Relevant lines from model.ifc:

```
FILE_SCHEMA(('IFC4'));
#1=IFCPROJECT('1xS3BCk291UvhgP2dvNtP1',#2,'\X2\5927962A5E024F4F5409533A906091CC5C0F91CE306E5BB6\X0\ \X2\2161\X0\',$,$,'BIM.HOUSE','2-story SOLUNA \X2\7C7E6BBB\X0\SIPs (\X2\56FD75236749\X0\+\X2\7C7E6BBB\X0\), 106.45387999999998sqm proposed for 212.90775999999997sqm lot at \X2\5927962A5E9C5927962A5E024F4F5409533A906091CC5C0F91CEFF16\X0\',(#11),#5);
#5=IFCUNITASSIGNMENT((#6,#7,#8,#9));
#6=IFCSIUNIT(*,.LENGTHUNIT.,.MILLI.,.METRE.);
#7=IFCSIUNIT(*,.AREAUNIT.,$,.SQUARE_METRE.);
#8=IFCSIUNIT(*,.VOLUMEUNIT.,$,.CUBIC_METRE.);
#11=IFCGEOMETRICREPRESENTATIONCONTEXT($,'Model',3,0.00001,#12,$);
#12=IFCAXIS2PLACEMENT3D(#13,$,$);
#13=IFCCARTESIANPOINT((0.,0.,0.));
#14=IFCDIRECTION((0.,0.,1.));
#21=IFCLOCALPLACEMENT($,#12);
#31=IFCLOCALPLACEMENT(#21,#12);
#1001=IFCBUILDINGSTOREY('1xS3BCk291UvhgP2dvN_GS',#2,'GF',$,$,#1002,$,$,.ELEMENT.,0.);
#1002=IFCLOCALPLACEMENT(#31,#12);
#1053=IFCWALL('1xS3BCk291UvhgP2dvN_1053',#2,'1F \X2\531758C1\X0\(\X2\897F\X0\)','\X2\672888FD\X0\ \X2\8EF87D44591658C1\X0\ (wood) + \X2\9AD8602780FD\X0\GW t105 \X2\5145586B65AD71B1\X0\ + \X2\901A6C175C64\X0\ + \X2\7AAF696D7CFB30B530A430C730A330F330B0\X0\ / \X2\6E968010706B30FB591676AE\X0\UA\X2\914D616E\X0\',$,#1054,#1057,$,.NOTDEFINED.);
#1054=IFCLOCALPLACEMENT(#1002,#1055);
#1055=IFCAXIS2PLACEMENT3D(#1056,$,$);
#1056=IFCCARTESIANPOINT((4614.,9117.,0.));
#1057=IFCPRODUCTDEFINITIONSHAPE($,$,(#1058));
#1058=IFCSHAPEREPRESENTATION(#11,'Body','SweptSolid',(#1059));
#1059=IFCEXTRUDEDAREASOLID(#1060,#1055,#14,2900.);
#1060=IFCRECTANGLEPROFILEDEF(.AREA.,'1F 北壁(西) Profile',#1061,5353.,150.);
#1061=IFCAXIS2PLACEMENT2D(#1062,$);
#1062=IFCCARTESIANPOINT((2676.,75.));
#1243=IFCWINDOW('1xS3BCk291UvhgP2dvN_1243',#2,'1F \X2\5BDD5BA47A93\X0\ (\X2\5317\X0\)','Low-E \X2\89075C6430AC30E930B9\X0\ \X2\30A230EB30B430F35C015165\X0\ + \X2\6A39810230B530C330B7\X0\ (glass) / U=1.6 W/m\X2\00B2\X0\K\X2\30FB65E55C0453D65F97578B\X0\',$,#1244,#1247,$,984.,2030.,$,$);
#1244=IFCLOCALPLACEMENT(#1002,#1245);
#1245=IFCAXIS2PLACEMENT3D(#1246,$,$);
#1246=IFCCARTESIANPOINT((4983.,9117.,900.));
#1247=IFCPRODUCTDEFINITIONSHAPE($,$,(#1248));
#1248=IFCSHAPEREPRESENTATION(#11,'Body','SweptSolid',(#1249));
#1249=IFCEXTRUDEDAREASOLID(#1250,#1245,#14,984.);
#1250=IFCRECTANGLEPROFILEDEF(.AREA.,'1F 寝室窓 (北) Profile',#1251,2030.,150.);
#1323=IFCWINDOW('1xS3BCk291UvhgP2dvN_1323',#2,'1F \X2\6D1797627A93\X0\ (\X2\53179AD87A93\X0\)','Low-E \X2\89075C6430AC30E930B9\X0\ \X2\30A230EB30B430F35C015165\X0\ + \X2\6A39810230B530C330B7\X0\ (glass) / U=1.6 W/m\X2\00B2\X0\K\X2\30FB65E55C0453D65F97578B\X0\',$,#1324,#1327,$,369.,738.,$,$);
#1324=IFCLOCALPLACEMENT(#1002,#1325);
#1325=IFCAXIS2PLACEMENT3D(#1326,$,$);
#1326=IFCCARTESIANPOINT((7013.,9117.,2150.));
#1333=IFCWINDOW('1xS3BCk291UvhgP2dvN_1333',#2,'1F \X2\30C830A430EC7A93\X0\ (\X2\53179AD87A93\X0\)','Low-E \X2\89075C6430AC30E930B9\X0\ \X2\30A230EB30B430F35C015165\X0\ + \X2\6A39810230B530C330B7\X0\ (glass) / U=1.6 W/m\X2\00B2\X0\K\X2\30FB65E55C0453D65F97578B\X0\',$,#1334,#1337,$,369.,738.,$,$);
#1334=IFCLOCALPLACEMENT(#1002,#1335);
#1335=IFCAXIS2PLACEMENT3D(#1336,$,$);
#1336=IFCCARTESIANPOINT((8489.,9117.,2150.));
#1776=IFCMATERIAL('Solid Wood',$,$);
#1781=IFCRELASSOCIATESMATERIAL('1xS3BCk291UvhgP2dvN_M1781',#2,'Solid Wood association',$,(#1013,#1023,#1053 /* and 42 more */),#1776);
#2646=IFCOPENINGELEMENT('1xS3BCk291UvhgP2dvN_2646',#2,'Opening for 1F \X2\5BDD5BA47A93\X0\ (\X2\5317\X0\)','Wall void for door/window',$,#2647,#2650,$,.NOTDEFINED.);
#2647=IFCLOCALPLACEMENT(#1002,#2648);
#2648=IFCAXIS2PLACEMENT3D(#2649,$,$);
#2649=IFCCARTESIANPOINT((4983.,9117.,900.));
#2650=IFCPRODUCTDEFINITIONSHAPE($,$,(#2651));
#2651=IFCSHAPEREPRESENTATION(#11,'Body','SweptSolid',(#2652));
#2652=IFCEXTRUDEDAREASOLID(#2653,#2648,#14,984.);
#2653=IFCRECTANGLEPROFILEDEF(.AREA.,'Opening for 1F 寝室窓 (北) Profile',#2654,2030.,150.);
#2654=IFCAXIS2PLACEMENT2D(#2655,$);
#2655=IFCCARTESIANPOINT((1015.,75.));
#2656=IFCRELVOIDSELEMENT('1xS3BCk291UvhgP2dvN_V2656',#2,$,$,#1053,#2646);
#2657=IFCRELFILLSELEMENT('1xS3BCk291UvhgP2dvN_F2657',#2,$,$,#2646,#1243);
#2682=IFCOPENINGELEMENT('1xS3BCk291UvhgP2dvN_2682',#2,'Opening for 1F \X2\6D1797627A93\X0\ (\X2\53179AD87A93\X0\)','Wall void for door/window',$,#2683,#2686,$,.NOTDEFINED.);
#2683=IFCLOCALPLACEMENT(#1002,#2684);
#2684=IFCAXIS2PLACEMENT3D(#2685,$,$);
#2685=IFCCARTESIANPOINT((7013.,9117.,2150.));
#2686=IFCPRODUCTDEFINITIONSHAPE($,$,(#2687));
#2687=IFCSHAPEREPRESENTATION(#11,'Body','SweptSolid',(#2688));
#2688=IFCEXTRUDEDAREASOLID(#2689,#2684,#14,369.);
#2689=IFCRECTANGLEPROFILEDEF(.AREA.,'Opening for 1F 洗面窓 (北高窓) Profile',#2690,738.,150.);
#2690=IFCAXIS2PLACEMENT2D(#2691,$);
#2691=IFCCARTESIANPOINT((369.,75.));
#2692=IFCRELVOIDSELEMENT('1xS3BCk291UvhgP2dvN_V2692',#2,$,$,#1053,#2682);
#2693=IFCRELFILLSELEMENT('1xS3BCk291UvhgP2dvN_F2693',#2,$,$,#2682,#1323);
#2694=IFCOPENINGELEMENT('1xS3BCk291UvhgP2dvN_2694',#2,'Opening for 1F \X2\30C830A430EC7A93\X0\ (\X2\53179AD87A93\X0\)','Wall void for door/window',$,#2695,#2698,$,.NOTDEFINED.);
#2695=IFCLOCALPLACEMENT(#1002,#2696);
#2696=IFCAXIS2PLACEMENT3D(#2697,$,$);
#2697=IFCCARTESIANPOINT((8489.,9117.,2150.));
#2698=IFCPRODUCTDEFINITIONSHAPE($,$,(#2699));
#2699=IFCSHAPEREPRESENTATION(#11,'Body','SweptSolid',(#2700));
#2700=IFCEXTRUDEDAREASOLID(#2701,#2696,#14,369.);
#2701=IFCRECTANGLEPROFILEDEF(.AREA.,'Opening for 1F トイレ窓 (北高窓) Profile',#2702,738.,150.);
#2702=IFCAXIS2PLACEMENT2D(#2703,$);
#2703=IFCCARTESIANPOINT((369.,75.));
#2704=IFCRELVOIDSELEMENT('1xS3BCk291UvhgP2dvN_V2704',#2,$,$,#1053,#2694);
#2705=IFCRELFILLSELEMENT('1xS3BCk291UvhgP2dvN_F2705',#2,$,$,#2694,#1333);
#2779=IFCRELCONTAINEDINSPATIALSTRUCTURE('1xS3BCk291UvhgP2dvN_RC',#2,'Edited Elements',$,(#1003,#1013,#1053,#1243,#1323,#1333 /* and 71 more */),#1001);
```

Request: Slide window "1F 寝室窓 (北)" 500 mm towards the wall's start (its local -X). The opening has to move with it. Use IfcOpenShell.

```python
import ifcopenshell
import ifcopenshell.api.geometry
import ifcopenshell.util.placement
import ifcopenshell.util.unit

model = ifcopenshell.open("model.ifc")
unit_scale = ifcopenshell.util.unit.calculate_unit_scale(model)

window = model.by_guid("1xS3BCk291UvhgP2dvN_1243")
opening = window.FillsVoids[0].RelatingOpeningElement
wall = opening.VoidsElements[0].RelatingBuildingElement

wall_matrix = ifcopenshell.util.placement.get_local_placement(wall.ObjectPlacement)
shift = wall_matrix[:3, 0] * -0.5 / unit_scale
before = ifcopenshell.util.placement.get_local_placement(window.ObjectPlacement)[:3, 3].copy()

# The window is not placed relative to its opening, so move both.
for product in (opening, window):
    matrix = ifcopenshell.util.placement.get_local_placement(product.ObjectPlacement)
    matrix[:3, 3] += shift
    ifcopenshell.api.geometry.edit_object_placement(model, product=product, matrix=matrix, is_si=False)

after = ifcopenshell.util.placement.get_local_placement(window.ObjectPlacement)[:3, 3]
print("window moved by", (after - before).round(3) + 0.0)

model.write("model-out.ifc")
```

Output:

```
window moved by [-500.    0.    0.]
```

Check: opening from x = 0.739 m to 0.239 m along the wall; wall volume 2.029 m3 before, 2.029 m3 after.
